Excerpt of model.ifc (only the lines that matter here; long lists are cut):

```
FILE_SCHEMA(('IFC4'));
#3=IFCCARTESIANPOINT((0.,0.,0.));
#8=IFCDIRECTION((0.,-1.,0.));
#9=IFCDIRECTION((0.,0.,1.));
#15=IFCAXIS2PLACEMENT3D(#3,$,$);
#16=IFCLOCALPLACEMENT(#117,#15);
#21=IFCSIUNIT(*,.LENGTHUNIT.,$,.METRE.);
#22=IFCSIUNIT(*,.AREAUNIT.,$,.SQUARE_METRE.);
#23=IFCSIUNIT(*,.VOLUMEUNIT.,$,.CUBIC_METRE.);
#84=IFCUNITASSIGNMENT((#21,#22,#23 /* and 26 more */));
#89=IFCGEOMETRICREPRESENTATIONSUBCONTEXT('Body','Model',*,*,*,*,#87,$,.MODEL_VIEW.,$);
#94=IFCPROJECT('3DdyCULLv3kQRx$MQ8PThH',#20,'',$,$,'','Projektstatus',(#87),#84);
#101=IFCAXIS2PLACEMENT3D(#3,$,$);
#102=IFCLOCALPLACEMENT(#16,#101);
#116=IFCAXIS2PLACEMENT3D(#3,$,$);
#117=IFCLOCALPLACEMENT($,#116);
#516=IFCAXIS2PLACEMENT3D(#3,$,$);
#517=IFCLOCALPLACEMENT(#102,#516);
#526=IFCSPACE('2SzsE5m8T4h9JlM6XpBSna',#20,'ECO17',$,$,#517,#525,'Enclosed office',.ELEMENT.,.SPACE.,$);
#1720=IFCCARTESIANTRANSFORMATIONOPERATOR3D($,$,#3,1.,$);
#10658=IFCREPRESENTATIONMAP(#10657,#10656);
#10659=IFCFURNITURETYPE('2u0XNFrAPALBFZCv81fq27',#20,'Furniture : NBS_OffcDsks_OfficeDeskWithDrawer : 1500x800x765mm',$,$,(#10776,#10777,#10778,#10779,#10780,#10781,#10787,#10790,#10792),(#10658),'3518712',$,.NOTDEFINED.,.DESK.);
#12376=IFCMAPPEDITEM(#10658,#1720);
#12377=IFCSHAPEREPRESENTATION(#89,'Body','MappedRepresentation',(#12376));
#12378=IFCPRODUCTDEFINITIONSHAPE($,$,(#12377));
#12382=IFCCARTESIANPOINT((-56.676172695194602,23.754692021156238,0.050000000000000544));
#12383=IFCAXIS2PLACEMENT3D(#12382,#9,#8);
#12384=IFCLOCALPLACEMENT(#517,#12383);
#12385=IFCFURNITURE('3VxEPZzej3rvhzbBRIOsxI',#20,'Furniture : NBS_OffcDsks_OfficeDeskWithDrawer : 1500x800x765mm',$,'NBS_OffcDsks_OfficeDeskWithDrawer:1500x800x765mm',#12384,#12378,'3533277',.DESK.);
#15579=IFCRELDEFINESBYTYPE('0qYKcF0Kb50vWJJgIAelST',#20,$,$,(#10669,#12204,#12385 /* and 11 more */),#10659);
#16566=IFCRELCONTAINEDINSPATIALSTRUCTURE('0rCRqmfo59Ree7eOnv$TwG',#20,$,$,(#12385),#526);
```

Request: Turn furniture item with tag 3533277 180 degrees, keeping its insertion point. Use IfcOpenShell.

```python
import ifcopenshell
import ifcopenshell.api.geometry
import ifcopenshell.util.placement

model = ifcopenshell.open("model.ifc")

item = model.by_id(12385)
matrix = ifcopenshell.util.placement.get_local_placement(item.ObjectPlacement)
matrix = matrix @ ifcopenshell.util.placement.rotation(180, "Z")
ifcopenshell.api.geometry.edit_object_placement(model, product=item, matrix=matrix, is_si=False)

print(ifcopenshell.util.placement.get_local_placement(item.ObjectPlacement).round(3) + 0.0)

model.write("model_edited.ifc")
```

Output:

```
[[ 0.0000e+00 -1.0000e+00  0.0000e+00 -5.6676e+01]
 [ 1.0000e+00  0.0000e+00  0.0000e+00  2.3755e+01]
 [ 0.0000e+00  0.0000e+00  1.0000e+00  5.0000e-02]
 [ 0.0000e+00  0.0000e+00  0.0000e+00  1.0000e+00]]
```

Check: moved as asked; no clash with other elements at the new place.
